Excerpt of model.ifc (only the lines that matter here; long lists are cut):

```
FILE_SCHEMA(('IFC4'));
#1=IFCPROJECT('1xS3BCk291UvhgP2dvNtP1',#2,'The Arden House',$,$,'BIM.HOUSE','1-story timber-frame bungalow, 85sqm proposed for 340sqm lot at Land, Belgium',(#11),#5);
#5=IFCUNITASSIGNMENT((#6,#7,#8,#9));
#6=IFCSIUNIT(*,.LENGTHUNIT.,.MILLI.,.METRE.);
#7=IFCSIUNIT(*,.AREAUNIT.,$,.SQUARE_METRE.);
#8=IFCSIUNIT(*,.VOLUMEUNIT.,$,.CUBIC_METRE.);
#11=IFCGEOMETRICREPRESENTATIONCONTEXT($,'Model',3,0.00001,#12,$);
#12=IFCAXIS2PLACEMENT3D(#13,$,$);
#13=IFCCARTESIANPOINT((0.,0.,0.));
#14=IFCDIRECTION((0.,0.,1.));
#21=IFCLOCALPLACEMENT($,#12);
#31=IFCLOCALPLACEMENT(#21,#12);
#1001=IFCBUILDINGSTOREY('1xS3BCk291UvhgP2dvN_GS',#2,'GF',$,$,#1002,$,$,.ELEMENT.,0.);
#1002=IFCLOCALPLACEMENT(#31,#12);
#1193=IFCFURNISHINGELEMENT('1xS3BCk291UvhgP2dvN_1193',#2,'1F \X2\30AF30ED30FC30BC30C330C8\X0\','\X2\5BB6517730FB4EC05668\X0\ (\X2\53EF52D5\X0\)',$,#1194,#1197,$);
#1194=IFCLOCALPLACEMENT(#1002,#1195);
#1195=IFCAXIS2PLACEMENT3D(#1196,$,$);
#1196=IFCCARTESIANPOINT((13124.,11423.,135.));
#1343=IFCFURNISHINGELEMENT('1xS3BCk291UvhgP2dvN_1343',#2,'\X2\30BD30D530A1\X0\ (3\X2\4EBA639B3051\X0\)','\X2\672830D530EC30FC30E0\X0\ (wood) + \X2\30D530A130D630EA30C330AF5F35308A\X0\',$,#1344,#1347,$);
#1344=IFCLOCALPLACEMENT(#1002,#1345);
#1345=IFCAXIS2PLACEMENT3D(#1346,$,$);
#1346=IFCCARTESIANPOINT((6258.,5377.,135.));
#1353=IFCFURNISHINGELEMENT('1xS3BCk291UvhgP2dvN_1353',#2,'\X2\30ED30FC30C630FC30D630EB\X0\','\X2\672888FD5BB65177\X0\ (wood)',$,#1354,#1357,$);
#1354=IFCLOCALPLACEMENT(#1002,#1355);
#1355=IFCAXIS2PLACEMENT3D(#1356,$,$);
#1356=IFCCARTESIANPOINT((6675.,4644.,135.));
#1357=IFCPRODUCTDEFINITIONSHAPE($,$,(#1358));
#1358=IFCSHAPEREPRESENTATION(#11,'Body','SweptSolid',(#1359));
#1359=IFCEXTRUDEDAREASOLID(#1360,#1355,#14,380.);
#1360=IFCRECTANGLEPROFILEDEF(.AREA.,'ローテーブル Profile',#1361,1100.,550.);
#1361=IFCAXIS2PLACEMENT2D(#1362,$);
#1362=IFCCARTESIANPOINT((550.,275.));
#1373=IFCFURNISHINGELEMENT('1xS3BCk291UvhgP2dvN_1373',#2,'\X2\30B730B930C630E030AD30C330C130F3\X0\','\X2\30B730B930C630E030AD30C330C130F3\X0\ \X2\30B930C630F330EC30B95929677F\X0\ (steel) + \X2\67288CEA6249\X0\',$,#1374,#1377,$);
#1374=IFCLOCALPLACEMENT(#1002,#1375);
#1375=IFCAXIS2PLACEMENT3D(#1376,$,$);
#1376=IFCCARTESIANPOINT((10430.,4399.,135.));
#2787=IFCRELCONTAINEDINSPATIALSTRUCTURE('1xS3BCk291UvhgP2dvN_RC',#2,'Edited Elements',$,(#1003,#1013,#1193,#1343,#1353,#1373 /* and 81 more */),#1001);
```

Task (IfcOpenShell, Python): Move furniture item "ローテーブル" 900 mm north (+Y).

```python
import ifcopenshell
import ifcopenshell.api.geometry
import ifcopenshell.util.placement
import ifcopenshell.util.unit

model = ifcopenshell.open("model.ifc")
unit_scale = ifcopenshell.util.unit.calculate_unit_scale(model)

item = model.by_id(1353)
matrix = ifcopenshell.util.placement.get_local_placement(item.ObjectPlacement)
matrix[1, 3] += 0.9 / unit_scale
ifcopenshell.api.geometry.edit_object_placement(model, product=item, matrix=matrix, is_si=False)

print(ifcopenshell.util.placement.get_local_placement(item.ObjectPlacement).round(3) + 0.0)

model.write("model-out.ifc")
```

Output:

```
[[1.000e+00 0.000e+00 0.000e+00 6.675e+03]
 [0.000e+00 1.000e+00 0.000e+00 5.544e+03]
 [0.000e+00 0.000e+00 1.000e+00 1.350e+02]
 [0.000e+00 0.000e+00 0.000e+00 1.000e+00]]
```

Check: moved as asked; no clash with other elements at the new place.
